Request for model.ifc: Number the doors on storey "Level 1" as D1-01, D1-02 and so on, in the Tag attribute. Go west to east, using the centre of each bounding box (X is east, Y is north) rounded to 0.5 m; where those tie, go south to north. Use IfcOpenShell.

First a look at what the model holds.

```python
import ifcopenshell
import ifcopenshell.util.element
import ifcopenshell.util.placement

model = ifcopenshell.open("model.ifc")
print(model.schema)
storey = next(s for s in model.by_type("IfcBuildingStorey") if s.Name == "Level 1")
doors = [e for e in ifcopenshell.util.element.get_decomposition(storey) if e.is_a("IfcDoor")]
for e in sorted(doors, key=lambda e: e.id()):
    origin = ifcopenshell.util.placement.get_local_placement(e.ObjectPlacement)[:3, 3]
    print(e.id(), e.Tag, e.Name, origin.round(2) + 0.0, sep=" | ")
```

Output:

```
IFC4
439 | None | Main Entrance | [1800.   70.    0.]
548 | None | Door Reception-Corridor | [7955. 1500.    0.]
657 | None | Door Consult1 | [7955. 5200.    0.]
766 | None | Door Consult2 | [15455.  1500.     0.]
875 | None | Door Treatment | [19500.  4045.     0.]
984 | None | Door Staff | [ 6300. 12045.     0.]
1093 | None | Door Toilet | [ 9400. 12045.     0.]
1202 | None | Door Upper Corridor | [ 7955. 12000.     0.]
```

```python
import ifcopenshell
import ifcopenshell.geom
import ifcopenshell.util.element
import ifcopenshell.util.shape

model = ifcopenshell.open("model.ifc")
settings = ifcopenshell.geom.settings()
settings.set("use-world-coords", True)


def centre(element):
    shape = ifcopenshell.geom.create_shape(settings, element)
    return ifcopenshell.util.shape.get_bbox_centroid(shape.geometry)


storey = next(s for s in model.by_type("IfcBuildingStorey") if s.Name == "Level 1")
doors = [e for e in ifcopenshell.util.element.get_decomposition(storey) if e.is_a("IfcDoor")]

# Insertion points can sit at a corner or the storey origin, so sort by the geometry (in metres).
centres = {e: centre(e) for e in doors}
doors.sort(key=lambda e: (round(centres[e][0] / 0.5), centres[e][1]))

for i, e in enumerate(doors, start=1):
    number = f"D1-{i:02d}"
    e.Tag = number
    print(e.id(), number)

model.write("model_updated.ifc")
```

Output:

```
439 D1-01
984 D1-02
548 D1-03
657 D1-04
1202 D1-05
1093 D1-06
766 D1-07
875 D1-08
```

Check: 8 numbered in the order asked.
